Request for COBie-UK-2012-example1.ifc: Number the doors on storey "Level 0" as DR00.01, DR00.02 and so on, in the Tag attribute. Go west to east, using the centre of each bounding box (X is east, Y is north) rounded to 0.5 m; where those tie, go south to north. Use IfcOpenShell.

First a look at what the model holds.

```python
import ifcopenshell
import ifcopenshell.util.element
import ifcopenshell.util.placement

model = ifcopenshell.open("COBie-UK-2012-example1.ifc")
print(model.schema)
storey = next(s for s in model.by_type("IfcBuildingStorey") if s.Name == "Level 0")
doors = [e for e in ifcopenshell.util.element.get_decomposition(storey) if e.is_a("IfcDoor")]
for e in sorted(doors, key=lambda e: e.id()):
    origin = ifcopenshell.util.placement.get_local_placement(e.ObjectPlacement)[:3, 3]
    print(e.id(), e.Tag, e.Name, origin.round(2) + 0.0, sep=" | ")
```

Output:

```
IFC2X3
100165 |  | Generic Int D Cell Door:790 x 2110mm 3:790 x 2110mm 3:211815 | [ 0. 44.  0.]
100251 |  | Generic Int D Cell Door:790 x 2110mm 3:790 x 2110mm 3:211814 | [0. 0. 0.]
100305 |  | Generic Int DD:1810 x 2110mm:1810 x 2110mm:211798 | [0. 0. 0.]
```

```python
import ifcopenshell
import ifcopenshell.geom
import ifcopenshell.util.element
import ifcopenshell.util.shape

model = ifcopenshell.open("COBie-UK-2012-example1.ifc")
settings = ifcopenshell.geom.settings()
settings.set("use-world-coords", True)


def centre(element):
    shape = ifcopenshell.geom.create_shape(settings, element)
    return ifcopenshell.util.shape.get_bbox_centroid(shape.geometry)


storey = next(s for s in model.by_type("IfcBuildingStorey") if s.Name == "Level 0")
doors = [e for e in ifcopenshell.util.element.get_decomposition(storey) if e.is_a("IfcDoor")]

# Insertion points can sit at a corner or the storey origin, so sort by the geometry (in metres).
centres = {e: centre(e) for e in doors}
doors.sort(key=lambda e: (round(centres[e][0] / 0.5), centres[e][1]))

for i, e in enumerate(doors, start=1):
    number = f"DR00.{i:02d}"
    e.Tag = number
    print(e.id(), number)

model.write("COBie-UK-2012-example1_updated.ifc")
```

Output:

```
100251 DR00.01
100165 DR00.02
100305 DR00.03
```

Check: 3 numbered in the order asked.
